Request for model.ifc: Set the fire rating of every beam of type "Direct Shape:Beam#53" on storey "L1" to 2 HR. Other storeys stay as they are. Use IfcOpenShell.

First a look at what the model holds.

```python
import ifcopenshell
import ifcopenshell.util.element

model = ifcopenshell.open("model.ifc")
print(model.schema)
storey = next(s for s in model.by_type("IfcBuildingStorey") if s.Name == "L1")
beams = [e for e in ifcopenshell.util.element.get_decomposition(storey) if e.is_a("IfcBeam")]
seen = {}
for e in beams:
    element_type = ifcopenshell.util.element.get_type(e)
    key = (element_type.Name if element_type != e and element_type else None, ifcopenshell.util.element.get_pset(e, "Pset_BeamCommon", "FireRating"))
    seen[key] = seen.get(key, 0) + 1
for (name, value), count in sorted(seen.items(), key=str):
    print(count, "x", name, "|", value)
```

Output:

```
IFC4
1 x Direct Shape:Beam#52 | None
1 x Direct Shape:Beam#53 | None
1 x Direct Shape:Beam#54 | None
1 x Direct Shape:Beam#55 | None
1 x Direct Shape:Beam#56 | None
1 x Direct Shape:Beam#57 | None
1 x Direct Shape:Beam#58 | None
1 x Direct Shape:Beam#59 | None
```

```python
import ifcopenshell
import ifcopenshell.api.pset
import ifcopenshell.util.element

model = ifcopenshell.open("model.ifc")

storey = next(s for s in model.by_type("IfcBuildingStorey") if s.Name == "L1")
beams = [e for e in ifcopenshell.util.element.get_decomposition(storey) if e.is_a("IfcBeam")]

count = 0
for e in beams:
    element_type = ifcopenshell.util.element.get_type(e)
    if element_type in (None, e) or element_type.Name != "Direct Shape:Beam#53":
        continue
    # add_pset returns the element's existing set when there is one.
    pset = ifcopenshell.api.pset.add_pset(model, product=e, name="Pset_BeamCommon")
    ifcopenshell.api.pset.edit_pset(model, pset=pset, properties={"FireRating": "2 HR"})
    count += 1

print(count, "beams updated")

model.write("model-out.ifc")
```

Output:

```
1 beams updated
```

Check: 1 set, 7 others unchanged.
